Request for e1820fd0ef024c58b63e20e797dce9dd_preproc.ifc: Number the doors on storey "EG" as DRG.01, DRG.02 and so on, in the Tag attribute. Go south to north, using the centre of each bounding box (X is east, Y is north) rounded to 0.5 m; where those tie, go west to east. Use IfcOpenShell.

First a look at what the model holds.

```python
import ifcopenshell
import ifcopenshell.util.element
import ifcopenshell.util.placement

model = ifcopenshell.open("e1820fd0ef024c58b63e20e797dce9dd_preproc.ifc")
print(model.schema)
storey = next(s for s in model.by_type("IfcBuildingStorey") if s.Name == "EG")
doors = [e for e in ifcopenshell.util.element.get_decomposition(storey) if e.is_a("IfcDoor")]
for e in sorted(doors, key=lambda e: e.id()):
    origin = ifcopenshell.util.placement.get_local_placement(e.ObjectPlacement)[:3, 3]
    print(e.id(), e.Tag, e.Name, origin.round(2) + 0.0, sep=" | ")
```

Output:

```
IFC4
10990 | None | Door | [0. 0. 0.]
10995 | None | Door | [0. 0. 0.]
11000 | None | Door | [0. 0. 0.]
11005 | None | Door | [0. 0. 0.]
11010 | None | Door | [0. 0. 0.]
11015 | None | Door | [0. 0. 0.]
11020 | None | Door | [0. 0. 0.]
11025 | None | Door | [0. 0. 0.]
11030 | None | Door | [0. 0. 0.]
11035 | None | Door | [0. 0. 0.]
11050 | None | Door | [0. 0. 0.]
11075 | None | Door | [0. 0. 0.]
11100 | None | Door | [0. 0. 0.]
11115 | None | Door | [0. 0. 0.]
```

```python
import ifcopenshell
import ifcopenshell.geom
import ifcopenshell.util.element
import ifcopenshell.util.shape

model = ifcopenshell.open("e1820fd0ef024c58b63e20e797dce9dd_preproc.ifc")
settings = ifcopenshell.geom.settings()
settings.set("use-world-coords", True)


def centre(element):
    shape = ifcopenshell.geom.create_shape(settings, element)
    return ifcopenshell.util.shape.get_bbox_centroid(shape.geometry)


storey = next(s for s in model.by_type("IfcBuildingStorey") if s.Name == "EG")
doors = [e for e in ifcopenshell.util.element.get_decomposition(storey) if e.is_a("IfcDoor")]

# Insertion points can sit at a corner or the storey origin, so sort by the geometry (in metres).
centres = {e: centre(e) for e in doors}
doors.sort(key=lambda e: (round(centres[e][1] / 0.5), centres[e][0]))

for i, e in enumerate(doors, start=1):
    number = f"DRG.{i:02d}"
    e.Tag = number
    print(e.id(), number)

model.write("e1820fd0ef024c58b63e20e797dce9dd_preproc_v2.ifc")
```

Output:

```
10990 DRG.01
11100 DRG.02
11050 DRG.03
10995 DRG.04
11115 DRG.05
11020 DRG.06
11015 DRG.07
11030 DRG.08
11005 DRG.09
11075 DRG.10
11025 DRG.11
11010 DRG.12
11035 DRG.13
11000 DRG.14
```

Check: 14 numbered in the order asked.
